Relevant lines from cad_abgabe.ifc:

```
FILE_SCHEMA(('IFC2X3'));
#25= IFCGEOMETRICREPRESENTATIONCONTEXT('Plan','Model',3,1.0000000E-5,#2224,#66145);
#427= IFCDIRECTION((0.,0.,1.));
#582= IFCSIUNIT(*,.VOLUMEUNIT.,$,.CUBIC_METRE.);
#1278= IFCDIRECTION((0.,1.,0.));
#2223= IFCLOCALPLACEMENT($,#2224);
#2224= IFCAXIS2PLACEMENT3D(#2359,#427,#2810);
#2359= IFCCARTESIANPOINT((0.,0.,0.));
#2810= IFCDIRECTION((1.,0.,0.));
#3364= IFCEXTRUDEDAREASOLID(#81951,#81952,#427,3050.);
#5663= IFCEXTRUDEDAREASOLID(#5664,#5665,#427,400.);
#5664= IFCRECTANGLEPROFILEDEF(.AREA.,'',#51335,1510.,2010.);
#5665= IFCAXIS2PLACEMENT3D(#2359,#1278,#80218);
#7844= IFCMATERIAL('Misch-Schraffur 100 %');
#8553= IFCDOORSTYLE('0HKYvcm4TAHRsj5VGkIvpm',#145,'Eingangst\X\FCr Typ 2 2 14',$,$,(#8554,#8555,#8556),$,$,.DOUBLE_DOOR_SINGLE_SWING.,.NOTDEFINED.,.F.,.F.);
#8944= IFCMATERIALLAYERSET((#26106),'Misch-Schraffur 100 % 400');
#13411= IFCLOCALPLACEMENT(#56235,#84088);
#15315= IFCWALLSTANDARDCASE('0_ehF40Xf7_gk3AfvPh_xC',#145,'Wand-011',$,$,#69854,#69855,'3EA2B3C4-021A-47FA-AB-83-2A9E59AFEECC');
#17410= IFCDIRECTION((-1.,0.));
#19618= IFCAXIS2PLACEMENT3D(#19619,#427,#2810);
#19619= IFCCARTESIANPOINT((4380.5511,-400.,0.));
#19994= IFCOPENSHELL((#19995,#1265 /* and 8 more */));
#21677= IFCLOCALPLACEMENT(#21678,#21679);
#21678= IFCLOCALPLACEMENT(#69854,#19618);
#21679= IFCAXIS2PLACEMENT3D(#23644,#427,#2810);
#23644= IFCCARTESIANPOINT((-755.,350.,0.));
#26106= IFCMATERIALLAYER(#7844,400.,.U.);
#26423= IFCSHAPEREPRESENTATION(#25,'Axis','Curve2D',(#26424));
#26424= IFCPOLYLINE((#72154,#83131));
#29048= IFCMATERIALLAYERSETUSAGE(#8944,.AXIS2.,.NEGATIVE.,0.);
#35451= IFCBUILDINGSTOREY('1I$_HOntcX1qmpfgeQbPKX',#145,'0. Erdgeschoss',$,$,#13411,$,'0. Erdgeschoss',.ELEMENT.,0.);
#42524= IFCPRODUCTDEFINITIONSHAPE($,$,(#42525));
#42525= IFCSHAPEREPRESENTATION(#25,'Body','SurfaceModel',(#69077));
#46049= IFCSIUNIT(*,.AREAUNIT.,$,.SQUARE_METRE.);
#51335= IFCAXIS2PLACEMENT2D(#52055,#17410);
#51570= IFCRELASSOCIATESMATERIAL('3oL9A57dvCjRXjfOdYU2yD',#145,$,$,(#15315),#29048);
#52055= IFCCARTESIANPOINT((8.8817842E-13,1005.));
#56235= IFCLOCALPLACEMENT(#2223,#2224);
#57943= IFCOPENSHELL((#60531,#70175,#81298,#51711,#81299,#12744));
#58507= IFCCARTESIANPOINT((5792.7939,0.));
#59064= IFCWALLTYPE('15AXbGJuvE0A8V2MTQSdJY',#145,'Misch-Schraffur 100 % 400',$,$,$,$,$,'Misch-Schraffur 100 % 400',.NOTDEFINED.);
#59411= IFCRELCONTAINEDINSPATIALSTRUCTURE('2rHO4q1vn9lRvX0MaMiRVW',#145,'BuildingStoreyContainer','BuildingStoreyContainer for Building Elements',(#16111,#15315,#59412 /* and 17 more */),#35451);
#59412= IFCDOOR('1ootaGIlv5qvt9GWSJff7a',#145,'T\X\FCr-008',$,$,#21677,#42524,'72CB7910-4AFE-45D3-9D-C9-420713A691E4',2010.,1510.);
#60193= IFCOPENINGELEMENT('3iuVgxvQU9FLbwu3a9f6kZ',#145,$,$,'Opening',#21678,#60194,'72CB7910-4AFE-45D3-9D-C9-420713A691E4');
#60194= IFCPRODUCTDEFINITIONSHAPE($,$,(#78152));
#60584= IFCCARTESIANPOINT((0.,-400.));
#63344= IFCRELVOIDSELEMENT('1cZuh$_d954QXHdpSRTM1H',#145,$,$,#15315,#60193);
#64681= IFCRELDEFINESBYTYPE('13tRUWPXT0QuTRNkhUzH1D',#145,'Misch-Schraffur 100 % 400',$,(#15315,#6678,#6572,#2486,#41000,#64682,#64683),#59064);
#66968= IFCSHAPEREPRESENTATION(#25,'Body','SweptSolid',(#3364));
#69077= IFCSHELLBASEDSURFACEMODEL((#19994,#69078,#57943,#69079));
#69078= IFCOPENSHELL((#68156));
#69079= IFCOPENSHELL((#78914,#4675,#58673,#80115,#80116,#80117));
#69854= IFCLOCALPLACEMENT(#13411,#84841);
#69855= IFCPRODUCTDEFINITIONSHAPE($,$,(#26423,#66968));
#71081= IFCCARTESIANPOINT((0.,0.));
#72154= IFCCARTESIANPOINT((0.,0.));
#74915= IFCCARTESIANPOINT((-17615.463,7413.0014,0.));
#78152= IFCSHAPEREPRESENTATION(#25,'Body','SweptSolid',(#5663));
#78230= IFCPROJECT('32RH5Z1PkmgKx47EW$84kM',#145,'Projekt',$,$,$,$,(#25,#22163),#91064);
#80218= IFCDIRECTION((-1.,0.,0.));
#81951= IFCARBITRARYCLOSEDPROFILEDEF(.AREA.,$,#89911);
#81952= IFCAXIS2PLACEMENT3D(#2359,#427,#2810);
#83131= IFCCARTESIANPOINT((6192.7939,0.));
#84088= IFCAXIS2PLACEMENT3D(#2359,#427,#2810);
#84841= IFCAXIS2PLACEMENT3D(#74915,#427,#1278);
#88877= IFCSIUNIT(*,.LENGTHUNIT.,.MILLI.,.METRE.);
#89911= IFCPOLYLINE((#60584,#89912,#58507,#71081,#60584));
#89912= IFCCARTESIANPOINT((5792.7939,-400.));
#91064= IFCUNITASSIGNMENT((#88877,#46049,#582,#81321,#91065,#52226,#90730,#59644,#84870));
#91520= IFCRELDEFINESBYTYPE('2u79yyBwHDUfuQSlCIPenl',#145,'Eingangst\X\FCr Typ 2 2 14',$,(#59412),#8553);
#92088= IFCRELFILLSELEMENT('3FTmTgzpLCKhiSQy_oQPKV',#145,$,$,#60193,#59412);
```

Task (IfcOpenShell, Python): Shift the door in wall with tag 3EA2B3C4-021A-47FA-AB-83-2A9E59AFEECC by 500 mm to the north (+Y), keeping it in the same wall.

```python
import ifcopenshell
import ifcopenshell.api.geometry
import ifcopenshell.util.placement

model = ifcopenshell.open("cad_abgabe.ifc")

door = model.by_id(59412)
opening = door.FillsVoids[0].RelatingOpeningElement
wall = opening.VoidsElements[0].RelatingBuildingElement

wall_matrix = ifcopenshell.util.placement.get_local_placement(wall.ObjectPlacement)
shift = wall_matrix[:3, 0] * 500.0
before = ifcopenshell.util.placement.get_local_placement(door.ObjectPlacement)[:3, 3].copy()

# The door is placed relative to its opening, so it follows when the opening moves.
matrix = ifcopenshell.util.placement.get_local_placement(opening.ObjectPlacement)
matrix[:3, 3] += shift
ifcopenshell.api.geometry.edit_object_placement(
    model, product=opening, matrix=matrix, is_si=False, should_transform_children=True
)

after = ifcopenshell.util.placement.get_local_placement(door.ObjectPlacement)[:3, 3]
print("door moved by", (after - before).round(3) + 0.0)

model.write("cad_abgabe_edited.ifc")
```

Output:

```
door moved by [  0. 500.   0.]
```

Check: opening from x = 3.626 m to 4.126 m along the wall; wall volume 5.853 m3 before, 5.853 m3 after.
